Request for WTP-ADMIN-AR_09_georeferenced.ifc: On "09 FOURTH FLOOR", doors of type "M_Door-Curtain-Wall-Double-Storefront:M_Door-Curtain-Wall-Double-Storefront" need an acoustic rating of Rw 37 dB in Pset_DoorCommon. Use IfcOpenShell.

First a look at what the model holds.

```python
import ifcopenshell
import ifcopenshell.util.element

model = ifcopenshell.open("WTP-ADMIN-AR_09_georeferenced.ifc")
print(model.schema)
storey = next(s for s in model.by_type("IfcBuildingStorey") if s.Name == "09 FOURTH FLOOR")
doors = [e for e in ifcopenshell.util.element.get_decomposition(storey) if e.is_a("IfcDoor")]
seen = {}
for e in doors:
    element_type = ifcopenshell.util.element.get_type(e)
    key = (element_type.Name if element_type != e and element_type else None, ifcopenshell.util.element.get_pset(e, "Pset_DoorCommon", "AcousticRating"))
    seen[key] = seen.get(key, 0) + 1
for (name, value), count in sorted(seen.items(), key=str):
    print(count, "x", name, "|", value)
```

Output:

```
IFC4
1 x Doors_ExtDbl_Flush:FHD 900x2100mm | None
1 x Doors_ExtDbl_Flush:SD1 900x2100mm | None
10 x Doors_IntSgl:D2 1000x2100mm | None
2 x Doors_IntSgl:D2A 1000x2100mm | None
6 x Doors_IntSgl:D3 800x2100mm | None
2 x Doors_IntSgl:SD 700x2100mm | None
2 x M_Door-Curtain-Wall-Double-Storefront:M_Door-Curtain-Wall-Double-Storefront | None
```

```python
import ifcopenshell
import ifcopenshell.api.pset
import ifcopenshell.util.element

model = ifcopenshell.open("WTP-ADMIN-AR_09_georeferenced.ifc")

storey = next(s for s in model.by_type("IfcBuildingStorey") if s.Name == "09 FOURTH FLOOR")
doors = [e for e in ifcopenshell.util.element.get_decomposition(storey) if e.is_a("IfcDoor")]

count = 0
for e in doors:
    element_type = ifcopenshell.util.element.get_type(e)
    if element_type in (None, e) or element_type.Name != "M_Door-Curtain-Wall-Double-Storefront:M_Door-Curtain-Wall-Double-Storefront":
        continue
    # add_pset returns the element's existing set when there is one.
    pset = ifcopenshell.api.pset.add_pset(model, product=e, name="Pset_DoorCommon")
    ifcopenshell.api.pset.edit_pset(model, pset=pset, properties={"AcousticRating": "Rw 37 dB"})
    count += 1

print(count, "doors updated")

model.write("WTP-ADMIN-AR_09_georeferenced_edited.ifc")
```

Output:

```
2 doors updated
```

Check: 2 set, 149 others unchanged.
